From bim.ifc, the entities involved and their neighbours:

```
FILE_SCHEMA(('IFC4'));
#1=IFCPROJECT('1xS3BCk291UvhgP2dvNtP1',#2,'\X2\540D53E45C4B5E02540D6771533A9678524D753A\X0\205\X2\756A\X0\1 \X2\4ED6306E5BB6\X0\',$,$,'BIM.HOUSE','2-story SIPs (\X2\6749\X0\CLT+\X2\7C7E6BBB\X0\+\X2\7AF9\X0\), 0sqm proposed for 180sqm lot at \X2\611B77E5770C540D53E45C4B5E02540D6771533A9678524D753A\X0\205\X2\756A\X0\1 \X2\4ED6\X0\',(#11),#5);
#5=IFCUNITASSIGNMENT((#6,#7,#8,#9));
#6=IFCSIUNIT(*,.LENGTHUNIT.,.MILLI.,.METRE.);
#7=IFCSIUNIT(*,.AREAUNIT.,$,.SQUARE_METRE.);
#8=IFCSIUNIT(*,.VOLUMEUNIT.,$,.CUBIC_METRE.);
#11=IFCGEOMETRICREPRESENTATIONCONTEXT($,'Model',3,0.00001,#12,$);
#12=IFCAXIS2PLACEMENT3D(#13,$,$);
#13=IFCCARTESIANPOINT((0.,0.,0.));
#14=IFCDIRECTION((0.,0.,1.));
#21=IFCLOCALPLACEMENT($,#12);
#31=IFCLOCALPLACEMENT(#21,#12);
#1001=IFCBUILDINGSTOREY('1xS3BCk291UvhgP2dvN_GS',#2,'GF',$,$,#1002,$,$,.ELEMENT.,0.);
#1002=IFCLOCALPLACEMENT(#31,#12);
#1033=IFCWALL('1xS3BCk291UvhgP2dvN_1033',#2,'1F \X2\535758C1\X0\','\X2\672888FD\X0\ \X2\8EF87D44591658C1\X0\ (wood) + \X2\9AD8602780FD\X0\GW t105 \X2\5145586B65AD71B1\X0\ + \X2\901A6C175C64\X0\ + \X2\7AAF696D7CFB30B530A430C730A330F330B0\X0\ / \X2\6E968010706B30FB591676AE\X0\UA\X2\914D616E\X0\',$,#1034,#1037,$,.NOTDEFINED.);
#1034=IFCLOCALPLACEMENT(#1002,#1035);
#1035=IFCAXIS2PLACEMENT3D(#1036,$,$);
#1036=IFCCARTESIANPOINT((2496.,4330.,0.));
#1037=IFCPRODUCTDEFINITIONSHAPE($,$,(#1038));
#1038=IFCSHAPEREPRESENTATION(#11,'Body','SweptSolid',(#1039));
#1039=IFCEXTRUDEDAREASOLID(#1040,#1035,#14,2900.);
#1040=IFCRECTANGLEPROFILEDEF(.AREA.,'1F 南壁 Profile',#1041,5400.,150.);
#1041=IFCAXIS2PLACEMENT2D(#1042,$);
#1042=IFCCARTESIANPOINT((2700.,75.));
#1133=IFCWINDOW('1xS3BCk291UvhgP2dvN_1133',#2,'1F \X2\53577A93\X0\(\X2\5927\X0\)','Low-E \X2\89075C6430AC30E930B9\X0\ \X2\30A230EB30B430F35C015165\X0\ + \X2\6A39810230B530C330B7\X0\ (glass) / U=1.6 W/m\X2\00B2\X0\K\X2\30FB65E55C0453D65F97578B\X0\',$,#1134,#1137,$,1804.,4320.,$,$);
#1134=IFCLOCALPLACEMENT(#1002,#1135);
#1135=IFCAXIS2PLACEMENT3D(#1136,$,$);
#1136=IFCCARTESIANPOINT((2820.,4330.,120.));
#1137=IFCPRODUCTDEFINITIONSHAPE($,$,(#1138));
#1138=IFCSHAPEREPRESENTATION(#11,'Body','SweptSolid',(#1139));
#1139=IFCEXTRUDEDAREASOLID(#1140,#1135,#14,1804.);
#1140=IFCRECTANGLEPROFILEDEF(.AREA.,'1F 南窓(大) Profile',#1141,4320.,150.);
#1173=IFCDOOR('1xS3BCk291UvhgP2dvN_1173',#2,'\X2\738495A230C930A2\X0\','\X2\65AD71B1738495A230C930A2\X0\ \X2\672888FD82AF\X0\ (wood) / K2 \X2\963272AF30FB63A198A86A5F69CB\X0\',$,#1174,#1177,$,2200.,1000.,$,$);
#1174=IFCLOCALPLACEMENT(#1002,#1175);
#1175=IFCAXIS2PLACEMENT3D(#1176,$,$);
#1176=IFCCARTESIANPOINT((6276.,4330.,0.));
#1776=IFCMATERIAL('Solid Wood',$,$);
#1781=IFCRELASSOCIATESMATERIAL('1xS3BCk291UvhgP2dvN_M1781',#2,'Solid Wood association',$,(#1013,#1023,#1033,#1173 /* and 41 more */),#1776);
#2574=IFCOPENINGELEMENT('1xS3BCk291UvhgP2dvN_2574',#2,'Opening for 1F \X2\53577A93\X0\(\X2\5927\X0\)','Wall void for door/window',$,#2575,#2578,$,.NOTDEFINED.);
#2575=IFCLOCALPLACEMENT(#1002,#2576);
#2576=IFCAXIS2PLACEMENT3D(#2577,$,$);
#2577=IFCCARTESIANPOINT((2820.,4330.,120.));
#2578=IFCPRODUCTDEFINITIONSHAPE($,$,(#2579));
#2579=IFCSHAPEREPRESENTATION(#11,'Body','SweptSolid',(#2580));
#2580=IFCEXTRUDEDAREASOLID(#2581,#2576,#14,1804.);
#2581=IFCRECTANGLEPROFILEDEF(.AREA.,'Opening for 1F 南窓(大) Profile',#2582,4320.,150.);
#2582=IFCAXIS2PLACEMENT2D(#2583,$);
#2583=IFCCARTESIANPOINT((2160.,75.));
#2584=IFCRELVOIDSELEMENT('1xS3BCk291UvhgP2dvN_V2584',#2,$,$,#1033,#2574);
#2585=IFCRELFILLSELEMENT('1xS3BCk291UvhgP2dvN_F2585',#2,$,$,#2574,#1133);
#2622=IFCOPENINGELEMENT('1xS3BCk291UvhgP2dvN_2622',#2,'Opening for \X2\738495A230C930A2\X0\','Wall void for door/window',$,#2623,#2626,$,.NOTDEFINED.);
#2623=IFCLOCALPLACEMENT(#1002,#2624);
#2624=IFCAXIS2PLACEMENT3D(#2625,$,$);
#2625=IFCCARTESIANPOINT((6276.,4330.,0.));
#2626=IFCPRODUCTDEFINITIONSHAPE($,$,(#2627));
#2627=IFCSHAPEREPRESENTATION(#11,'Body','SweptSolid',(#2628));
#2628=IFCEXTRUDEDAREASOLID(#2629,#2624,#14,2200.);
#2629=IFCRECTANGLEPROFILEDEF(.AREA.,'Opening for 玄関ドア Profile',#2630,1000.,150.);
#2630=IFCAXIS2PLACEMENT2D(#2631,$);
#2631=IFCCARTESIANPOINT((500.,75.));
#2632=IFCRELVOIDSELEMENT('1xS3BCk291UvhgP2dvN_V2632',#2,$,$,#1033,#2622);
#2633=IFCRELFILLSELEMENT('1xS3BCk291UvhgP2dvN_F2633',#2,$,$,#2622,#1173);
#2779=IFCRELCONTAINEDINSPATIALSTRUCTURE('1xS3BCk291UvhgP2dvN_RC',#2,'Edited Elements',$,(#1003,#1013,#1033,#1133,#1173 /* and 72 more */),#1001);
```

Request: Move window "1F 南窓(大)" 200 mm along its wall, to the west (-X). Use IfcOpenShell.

```python
import ifcopenshell
import ifcopenshell.api.geometry
import ifcopenshell.util.placement
import ifcopenshell.util.unit

model = ifcopenshell.open("bim.ifc")
unit_scale = ifcopenshell.util.unit.calculate_unit_scale(model)

window = model.by_id(1133)
opening = window.FillsVoids[0].RelatingOpeningElement
wall = opening.VoidsElements[0].RelatingBuildingElement

wall_matrix = ifcopenshell.util.placement.get_local_placement(wall.ObjectPlacement)
shift = wall_matrix[:3, 0] * -0.2 / unit_scale
before = ifcopenshell.util.placement.get_local_placement(window.ObjectPlacement)[:3, 3].copy()

# The window is not placed relative to its opening, so move both.
for product in (opening, window):
    matrix = ifcopenshell.util.placement.get_local_placement(product.ObjectPlacement)
    matrix[:3, 3] += shift
    ifcopenshell.api.geometry.edit_object_placement(model, product=product, matrix=matrix, is_si=False)

after = ifcopenshell.util.placement.get_local_placement(window.ObjectPlacement)[:3, 3]
print("window moved by", (after - before).round(3) + 0.0)

model.write("bim_rev.ifc")
```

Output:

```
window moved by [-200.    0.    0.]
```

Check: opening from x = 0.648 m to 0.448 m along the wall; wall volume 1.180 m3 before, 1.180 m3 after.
